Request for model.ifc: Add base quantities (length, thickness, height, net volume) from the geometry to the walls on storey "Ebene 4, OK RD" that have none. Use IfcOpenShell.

First a look at what the model holds.

```python
import ifcopenshell
import ifcopenshell.util.element
import ifcopenshell.util.unit

model = ifcopenshell.open("model.ifc")
print(model.schema)
for unit_type in ("LENGTHUNIT", "AREAUNIT", "VOLUMEUNIT"):
    print(unit_type, ifcopenshell.util.unit.calculate_unit_scale(model, unit_type))
storey = next(s for s in model.by_type("IfcBuildingStorey") if s.Name == "Ebene 4, OK RD")
walls = [e for e in ifcopenshell.util.element.get_decomposition(storey) if e.is_a("IfcWall")]
for e in sorted(walls, key=lambda e: e.id()):
    print(e.id(), e.is_a(), e.Name, list(ifcopenshell.util.element.get_psets(e, qtos_only=True)), sep=" | ")
```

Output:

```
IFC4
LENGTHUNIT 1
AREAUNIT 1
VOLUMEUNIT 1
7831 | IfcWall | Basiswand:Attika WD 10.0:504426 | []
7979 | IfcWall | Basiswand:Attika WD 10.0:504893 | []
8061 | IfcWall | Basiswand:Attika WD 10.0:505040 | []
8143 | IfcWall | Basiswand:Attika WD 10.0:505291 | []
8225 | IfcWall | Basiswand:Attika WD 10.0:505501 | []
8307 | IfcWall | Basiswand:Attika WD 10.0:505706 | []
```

```python
import ifcopenshell
import ifcopenshell.api.pset
import ifcopenshell.geom
import ifcopenshell.util.element
import ifcopenshell.util.shape
import ifcopenshell.util.unit

model = ifcopenshell.open("model.ifc")
unit_scale = ifcopenshell.util.unit.calculate_unit_scale(model)
volume_scale = ifcopenshell.util.unit.calculate_unit_scale(model, "VOLUMEUNIT")
settings = ifcopenshell.geom.settings()

storey = next(s for s in model.by_type("IfcBuildingStorey") if s.Name == "Ebene 4, OK RD")
walls = [e for e in ifcopenshell.util.element.get_decomposition(storey) if e.is_a("IfcWall")]

for e in sorted(walls, key=lambda e: e.id()):
    if ifcopenshell.util.element.get_psets(e, qtos_only=True, should_inherit=False):
        continue
    # Geometry comes back in metres, in the element's own axes.
    shape = ifcopenshell.geom.create_shape(settings, e)
    values = {
        "Length": ifcopenshell.util.shape.get_x(shape.geometry) / unit_scale,
        "Width": ifcopenshell.util.shape.get_y(shape.geometry) / unit_scale,
        "Height": ifcopenshell.util.shape.get_z(shape.geometry) / unit_scale,
        "NetVolume": ifcopenshell.util.shape.get_volume(shape.geometry) / volume_scale,
    }
    qto = ifcopenshell.api.pset.add_qto(model, product=e, name="Qto_WallBaseQuantities")
    ifcopenshell.api.pset.edit_qto(model, qto=qto, properties=values)
    print(e.id(), {k: round(v, 3) for k, v in values.items()})

model.write("model_rev.ifc")
```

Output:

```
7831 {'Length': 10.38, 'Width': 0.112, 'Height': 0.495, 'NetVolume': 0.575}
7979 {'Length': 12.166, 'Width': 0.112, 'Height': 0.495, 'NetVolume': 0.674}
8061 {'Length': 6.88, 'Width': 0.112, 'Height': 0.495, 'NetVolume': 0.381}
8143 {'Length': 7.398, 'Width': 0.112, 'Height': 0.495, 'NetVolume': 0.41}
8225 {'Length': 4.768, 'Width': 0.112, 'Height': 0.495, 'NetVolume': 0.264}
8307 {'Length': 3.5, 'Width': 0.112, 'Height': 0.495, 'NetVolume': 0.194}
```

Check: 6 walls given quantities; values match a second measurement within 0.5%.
